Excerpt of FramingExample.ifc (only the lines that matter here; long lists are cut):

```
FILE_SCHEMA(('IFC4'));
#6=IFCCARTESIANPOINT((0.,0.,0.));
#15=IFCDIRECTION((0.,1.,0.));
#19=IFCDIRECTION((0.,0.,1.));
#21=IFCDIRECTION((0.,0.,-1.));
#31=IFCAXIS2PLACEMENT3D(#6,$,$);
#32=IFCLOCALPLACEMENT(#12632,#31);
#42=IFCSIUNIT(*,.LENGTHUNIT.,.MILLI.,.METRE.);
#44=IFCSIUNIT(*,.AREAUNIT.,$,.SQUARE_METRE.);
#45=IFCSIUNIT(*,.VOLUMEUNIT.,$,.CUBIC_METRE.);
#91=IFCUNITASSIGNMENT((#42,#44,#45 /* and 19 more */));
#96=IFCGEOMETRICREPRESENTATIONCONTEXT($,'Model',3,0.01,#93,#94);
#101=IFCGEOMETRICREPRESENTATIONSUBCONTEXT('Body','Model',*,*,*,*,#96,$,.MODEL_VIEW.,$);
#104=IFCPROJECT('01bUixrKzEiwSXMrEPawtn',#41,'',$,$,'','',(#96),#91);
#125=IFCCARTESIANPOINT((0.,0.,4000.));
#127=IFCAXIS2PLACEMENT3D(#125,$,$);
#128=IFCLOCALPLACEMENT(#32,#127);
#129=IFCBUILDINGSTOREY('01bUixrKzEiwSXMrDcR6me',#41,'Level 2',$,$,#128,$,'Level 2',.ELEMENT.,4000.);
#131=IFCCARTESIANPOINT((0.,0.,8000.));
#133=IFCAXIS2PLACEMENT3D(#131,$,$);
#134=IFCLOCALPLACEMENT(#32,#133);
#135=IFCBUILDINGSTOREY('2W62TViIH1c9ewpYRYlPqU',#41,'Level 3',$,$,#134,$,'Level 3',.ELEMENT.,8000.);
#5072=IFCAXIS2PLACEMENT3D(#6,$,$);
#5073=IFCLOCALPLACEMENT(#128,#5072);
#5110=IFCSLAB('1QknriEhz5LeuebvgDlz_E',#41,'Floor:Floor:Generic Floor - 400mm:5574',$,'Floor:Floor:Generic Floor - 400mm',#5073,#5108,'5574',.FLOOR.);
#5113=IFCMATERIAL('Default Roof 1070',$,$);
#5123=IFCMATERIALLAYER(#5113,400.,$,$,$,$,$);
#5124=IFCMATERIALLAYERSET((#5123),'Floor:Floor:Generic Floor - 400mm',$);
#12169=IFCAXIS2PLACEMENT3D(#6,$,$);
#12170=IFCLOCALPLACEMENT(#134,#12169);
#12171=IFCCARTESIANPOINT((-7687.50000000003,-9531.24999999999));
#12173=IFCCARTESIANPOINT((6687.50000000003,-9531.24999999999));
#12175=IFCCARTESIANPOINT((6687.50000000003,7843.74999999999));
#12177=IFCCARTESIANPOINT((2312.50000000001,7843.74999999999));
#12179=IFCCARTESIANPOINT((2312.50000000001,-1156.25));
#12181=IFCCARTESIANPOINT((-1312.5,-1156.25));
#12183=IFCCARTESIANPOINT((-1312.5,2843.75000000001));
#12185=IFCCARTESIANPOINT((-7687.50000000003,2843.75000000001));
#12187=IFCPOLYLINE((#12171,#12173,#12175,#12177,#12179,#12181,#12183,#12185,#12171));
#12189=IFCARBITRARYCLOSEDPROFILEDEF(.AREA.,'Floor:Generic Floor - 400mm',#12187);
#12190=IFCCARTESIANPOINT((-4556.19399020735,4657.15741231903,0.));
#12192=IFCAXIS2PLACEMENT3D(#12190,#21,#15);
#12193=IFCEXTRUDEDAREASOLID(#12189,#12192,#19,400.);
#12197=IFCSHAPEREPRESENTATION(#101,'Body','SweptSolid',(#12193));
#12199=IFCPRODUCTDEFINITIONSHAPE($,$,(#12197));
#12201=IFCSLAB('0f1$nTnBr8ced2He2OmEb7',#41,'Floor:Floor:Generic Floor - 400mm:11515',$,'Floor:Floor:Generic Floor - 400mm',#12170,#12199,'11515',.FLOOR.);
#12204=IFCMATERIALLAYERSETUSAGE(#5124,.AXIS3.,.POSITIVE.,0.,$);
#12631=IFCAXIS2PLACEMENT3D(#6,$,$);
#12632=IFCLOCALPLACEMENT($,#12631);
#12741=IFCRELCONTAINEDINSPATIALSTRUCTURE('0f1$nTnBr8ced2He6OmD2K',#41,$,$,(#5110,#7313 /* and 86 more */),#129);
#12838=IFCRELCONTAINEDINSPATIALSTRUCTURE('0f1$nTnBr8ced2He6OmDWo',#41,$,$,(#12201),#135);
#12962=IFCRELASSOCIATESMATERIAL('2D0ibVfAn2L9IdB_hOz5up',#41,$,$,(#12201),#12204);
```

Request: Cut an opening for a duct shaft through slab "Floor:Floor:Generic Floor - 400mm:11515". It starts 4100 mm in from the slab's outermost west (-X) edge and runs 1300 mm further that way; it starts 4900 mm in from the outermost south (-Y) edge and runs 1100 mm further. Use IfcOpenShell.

```python
import numpy as np
import ifcopenshell
import ifcopenshell.api.feature
import ifcopenshell.api.geometry
import ifcopenshell.api.root
import ifcopenshell.geom
import ifcopenshell.util.placement
import ifcopenshell.util.representation
import ifcopenshell.util.shape
import ifcopenshell.util.unit

model = ifcopenshell.open("FramingExample.ifc")
unit_scale = ifcopenshell.util.unit.calculate_unit_scale(model)
settings = ifcopenshell.geom.settings()


def volume(element):
    """Net volume in cubic metres, openings subtracted."""
    shape = ifcopenshell.geom.create_shape(settings, element)
    return ifcopenshell.util.shape.get_volume(shape.geometry)


slab = model.by_id(12201)
before = volume(slab)

# Extent in the slab's own axes, in metres. The edges named are its -X and -Y sides.
slab_shape = ifcopenshell.geom.create_shape(settings, slab)
vertices = ifcopenshell.util.shape.get_vertices(slab_shape.geometry)
x_min, y_min, bottom = vertices.min(axis=0)
top = vertices[:, 2].max()

opening = ifcopenshell.api.root.create_entity(model, ifc_class="IfcOpeningElement", name="Duct shaft opening", predefined_type="OPENING")
context = ifcopenshell.util.representation.get_context(model, "Model", "Body", "MODEL_VIEW")
width, depth = 1.3, 1.1
outline = [(0.0, 0.0), (width, 0.0), (width, depth), (0.0, depth), (0.0, 0.0)]
# Overshoot both faces by 50 mm so the cut is clean.
shape = ifcopenshell.api.geometry.add_slab_representation(
    model, context=context, depth=top - bottom + 0.1, polyline=outline
)
ifcopenshell.api.geometry.assign_representation(model, product=opening, representation=shape)

matrix = ifcopenshell.util.placement.get_local_placement(slab.ObjectPlacement)
matrix[:, 3] = matrix @ np.append(np.array([x_min + 4.1, y_min + 4.9, bottom - 0.05]) / unit_scale, 1.0)
ifcopenshell.api.geometry.edit_object_placement(model, product=opening, matrix=matrix, is_si=False)
ifcopenshell.api.feature.add_feature(model, feature=opening, element=slab)

after = volume(slab)

print(f"slab volume {before:.3f} -> {after:.3f} m3")

model.write("FramingExample_v2.ifc")
```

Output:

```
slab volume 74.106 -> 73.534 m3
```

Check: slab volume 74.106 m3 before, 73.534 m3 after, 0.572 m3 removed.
